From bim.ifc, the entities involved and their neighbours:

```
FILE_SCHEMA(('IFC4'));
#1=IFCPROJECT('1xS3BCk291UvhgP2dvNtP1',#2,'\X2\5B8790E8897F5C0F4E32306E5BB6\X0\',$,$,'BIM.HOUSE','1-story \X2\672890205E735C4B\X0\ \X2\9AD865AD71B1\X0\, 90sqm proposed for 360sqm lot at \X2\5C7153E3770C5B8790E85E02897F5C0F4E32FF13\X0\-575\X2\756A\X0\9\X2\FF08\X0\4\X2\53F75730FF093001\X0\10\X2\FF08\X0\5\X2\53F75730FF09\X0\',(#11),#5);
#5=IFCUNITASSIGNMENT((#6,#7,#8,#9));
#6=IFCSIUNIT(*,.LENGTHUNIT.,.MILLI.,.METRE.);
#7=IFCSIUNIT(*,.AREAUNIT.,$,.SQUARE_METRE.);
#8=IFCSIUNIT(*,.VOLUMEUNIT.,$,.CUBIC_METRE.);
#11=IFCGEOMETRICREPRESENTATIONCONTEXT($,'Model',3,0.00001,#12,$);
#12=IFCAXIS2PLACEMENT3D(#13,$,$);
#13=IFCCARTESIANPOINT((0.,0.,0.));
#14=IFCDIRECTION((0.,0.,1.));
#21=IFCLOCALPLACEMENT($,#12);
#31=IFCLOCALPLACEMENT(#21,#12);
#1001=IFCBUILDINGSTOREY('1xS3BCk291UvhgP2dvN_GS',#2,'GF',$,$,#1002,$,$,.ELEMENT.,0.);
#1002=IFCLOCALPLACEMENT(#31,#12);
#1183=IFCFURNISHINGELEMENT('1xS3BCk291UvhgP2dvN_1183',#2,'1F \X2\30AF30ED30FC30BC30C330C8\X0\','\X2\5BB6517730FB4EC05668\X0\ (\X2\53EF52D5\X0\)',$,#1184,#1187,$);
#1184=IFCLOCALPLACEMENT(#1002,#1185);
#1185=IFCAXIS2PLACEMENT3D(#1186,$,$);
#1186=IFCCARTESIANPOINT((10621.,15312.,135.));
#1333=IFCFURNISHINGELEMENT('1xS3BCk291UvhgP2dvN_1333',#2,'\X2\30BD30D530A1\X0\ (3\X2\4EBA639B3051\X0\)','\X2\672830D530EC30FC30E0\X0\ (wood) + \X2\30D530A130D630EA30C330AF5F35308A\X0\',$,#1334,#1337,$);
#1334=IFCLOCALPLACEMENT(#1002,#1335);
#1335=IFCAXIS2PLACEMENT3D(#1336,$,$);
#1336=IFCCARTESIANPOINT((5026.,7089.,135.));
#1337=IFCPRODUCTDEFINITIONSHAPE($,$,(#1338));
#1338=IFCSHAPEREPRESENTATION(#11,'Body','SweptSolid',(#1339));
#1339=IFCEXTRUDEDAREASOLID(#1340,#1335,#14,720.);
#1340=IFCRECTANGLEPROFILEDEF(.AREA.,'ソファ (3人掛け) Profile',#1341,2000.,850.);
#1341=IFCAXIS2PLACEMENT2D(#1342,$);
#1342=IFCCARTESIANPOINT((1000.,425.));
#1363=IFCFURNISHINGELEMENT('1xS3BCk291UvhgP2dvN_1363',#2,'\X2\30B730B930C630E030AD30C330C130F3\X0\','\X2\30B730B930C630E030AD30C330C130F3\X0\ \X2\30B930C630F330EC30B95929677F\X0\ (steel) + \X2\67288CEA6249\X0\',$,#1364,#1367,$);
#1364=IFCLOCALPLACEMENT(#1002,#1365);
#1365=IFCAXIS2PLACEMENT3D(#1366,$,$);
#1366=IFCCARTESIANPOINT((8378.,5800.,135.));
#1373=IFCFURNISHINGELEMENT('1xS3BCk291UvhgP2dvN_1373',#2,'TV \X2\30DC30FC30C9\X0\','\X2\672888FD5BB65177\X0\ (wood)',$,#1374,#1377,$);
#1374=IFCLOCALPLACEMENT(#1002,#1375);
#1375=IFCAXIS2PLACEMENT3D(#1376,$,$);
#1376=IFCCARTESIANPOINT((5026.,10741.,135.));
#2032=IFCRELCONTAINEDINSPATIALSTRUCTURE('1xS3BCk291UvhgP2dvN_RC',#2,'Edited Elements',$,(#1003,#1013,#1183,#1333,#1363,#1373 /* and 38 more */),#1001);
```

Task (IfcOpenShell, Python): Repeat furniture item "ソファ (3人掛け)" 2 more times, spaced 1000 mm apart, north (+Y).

```python
import numpy as np
import ifcopenshell
import ifcopenshell.api.geometry
import ifcopenshell.api.root
import ifcopenshell.util.element
import ifcopenshell.util.placement

model = ifcopenshell.open("bim.ifc")


def reuse_history(source, copy):
    """copy_class also copies each property set's owner history, people and application; keep the originals."""
    for rel in copy.IsDefinedBy:
        if rel.is_a("IfcRelDefinesByProperties") and (history := rel.RelatingPropertyDefinition.OwnerHistory):
            rel.RelatingPropertyDefinition.OwnerHistory = source.OwnerHistory
            ifcopenshell.util.element.remove_deep2(model, history)


source = model.by_guid("1xS3BCk291UvhgP2dvN_1333")
base = ifcopenshell.util.placement.get_local_placement(source.ObjectPlacement)
step = np.array([0.0, 1.0, 0.0]) * 1000.0

for i in range(1, 3):
    copy = ifcopenshell.api.root.copy_class(model, product=source)
    copy.Representation = ifcopenshell.util.element.copy_deep(
        model, source.Representation, exclude=["IfcGeometricRepresentationContext", "IfcRepresentationMap"]
    )
    reuse_history(source, copy)
    matrix = base.copy()
    matrix[:3, 3] += i * step
    print("added at", matrix[:3, 3].round(3) + 0.0)
    ifcopenshell.api.geometry.edit_object_placement(model, product=copy, matrix=matrix, is_si=False)

model.write("bim_updated.ifc")
```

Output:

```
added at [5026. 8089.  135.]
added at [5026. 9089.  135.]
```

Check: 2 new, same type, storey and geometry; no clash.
